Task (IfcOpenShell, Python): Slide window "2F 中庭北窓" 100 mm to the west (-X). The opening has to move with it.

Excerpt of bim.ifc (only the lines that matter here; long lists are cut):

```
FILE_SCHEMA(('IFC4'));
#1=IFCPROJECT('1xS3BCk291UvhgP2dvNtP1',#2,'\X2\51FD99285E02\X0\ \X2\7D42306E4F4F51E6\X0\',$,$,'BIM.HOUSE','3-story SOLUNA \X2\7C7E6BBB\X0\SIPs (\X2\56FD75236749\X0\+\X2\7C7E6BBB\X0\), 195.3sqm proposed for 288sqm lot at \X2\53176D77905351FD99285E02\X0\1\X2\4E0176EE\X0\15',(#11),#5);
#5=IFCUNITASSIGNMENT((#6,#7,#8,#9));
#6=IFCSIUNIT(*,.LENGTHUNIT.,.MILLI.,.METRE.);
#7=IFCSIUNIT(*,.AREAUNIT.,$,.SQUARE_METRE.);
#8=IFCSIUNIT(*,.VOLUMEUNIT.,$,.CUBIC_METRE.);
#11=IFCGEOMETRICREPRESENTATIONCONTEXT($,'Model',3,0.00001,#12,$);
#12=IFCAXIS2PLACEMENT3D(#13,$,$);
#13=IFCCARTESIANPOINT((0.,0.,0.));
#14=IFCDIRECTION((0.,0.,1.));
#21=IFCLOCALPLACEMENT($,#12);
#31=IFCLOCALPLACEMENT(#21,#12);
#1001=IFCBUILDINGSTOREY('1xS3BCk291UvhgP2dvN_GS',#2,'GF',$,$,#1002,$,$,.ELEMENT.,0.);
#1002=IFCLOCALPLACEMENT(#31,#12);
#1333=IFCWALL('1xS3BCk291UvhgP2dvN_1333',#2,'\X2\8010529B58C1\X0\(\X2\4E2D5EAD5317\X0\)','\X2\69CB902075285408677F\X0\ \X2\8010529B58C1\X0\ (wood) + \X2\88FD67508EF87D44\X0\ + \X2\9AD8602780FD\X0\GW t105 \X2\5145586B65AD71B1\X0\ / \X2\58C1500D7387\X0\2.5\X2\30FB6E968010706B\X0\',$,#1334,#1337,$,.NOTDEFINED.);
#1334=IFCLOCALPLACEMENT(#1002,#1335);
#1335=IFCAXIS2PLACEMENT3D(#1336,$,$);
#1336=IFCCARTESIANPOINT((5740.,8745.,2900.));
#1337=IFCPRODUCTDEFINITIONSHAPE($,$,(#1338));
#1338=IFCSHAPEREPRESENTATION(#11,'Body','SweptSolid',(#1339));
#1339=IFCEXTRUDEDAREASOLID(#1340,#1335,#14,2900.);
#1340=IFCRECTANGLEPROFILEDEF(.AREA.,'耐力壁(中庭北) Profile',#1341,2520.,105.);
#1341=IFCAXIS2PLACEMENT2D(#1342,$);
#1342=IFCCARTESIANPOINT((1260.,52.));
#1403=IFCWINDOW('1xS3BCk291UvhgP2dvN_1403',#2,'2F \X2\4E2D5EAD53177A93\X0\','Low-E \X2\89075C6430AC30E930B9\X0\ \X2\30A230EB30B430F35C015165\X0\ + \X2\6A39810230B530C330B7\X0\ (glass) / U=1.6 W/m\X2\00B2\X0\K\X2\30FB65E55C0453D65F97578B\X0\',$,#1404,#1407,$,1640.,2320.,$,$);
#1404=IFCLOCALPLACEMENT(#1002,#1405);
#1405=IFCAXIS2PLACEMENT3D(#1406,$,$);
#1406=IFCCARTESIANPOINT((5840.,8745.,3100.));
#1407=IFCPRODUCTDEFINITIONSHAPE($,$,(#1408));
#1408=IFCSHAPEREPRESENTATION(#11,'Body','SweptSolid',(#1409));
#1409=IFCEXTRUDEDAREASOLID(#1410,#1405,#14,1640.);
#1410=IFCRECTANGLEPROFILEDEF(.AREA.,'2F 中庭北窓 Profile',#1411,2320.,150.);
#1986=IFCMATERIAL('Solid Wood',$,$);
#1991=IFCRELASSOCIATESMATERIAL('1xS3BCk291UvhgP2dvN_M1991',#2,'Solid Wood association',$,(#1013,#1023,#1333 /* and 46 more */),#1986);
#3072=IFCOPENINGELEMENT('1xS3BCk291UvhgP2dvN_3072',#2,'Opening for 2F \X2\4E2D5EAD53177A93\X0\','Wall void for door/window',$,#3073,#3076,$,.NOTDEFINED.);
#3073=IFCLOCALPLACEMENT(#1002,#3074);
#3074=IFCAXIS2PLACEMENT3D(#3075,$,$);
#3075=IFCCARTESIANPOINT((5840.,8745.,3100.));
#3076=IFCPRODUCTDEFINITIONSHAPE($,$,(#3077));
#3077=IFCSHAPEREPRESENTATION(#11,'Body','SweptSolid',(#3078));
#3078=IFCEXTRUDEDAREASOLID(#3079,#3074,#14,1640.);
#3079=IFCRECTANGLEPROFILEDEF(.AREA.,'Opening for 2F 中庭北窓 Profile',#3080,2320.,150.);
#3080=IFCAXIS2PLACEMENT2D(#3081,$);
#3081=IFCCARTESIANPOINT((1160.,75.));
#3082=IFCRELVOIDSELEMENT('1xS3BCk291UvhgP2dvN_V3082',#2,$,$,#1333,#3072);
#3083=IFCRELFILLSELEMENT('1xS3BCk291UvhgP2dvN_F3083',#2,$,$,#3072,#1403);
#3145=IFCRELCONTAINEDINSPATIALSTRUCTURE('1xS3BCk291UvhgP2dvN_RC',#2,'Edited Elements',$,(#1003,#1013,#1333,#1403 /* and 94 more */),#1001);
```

```python
import ifcopenshell
import ifcopenshell.api.geometry
import ifcopenshell.util.placement
import ifcopenshell.util.unit

model = ifcopenshell.open("bim.ifc")
unit_scale = ifcopenshell.util.unit.calculate_unit_scale(model)

window = model.by_guid("1xS3BCk291UvhgP2dvN_1403")
opening = window.FillsVoids[0].RelatingOpeningElement
wall = opening.VoidsElements[0].RelatingBuildingElement

wall_matrix = ifcopenshell.util.placement.get_local_placement(wall.ObjectPlacement)
shift = wall_matrix[:3, 0] * -0.1 / unit_scale
before = ifcopenshell.util.placement.get_local_placement(window.ObjectPlacement)[:3, 3].copy()

# The window is not placed relative to its opening, so move both.
for product in (opening, window):
    matrix = ifcopenshell.util.placement.get_local_placement(product.ObjectPlacement)
    matrix[:3, 3] += shift
    ifcopenshell.api.geometry.edit_object_placement(model, product=product, matrix=matrix, is_si=False)

after = ifcopenshell.util.placement.get_local_placement(window.ObjectPlacement)[:3, 3]
print("window moved by", (after - before).round(3) + 0.0)

model.write("bim-out.ifc")
```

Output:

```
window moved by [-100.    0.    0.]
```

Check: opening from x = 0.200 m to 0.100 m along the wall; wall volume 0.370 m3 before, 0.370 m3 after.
